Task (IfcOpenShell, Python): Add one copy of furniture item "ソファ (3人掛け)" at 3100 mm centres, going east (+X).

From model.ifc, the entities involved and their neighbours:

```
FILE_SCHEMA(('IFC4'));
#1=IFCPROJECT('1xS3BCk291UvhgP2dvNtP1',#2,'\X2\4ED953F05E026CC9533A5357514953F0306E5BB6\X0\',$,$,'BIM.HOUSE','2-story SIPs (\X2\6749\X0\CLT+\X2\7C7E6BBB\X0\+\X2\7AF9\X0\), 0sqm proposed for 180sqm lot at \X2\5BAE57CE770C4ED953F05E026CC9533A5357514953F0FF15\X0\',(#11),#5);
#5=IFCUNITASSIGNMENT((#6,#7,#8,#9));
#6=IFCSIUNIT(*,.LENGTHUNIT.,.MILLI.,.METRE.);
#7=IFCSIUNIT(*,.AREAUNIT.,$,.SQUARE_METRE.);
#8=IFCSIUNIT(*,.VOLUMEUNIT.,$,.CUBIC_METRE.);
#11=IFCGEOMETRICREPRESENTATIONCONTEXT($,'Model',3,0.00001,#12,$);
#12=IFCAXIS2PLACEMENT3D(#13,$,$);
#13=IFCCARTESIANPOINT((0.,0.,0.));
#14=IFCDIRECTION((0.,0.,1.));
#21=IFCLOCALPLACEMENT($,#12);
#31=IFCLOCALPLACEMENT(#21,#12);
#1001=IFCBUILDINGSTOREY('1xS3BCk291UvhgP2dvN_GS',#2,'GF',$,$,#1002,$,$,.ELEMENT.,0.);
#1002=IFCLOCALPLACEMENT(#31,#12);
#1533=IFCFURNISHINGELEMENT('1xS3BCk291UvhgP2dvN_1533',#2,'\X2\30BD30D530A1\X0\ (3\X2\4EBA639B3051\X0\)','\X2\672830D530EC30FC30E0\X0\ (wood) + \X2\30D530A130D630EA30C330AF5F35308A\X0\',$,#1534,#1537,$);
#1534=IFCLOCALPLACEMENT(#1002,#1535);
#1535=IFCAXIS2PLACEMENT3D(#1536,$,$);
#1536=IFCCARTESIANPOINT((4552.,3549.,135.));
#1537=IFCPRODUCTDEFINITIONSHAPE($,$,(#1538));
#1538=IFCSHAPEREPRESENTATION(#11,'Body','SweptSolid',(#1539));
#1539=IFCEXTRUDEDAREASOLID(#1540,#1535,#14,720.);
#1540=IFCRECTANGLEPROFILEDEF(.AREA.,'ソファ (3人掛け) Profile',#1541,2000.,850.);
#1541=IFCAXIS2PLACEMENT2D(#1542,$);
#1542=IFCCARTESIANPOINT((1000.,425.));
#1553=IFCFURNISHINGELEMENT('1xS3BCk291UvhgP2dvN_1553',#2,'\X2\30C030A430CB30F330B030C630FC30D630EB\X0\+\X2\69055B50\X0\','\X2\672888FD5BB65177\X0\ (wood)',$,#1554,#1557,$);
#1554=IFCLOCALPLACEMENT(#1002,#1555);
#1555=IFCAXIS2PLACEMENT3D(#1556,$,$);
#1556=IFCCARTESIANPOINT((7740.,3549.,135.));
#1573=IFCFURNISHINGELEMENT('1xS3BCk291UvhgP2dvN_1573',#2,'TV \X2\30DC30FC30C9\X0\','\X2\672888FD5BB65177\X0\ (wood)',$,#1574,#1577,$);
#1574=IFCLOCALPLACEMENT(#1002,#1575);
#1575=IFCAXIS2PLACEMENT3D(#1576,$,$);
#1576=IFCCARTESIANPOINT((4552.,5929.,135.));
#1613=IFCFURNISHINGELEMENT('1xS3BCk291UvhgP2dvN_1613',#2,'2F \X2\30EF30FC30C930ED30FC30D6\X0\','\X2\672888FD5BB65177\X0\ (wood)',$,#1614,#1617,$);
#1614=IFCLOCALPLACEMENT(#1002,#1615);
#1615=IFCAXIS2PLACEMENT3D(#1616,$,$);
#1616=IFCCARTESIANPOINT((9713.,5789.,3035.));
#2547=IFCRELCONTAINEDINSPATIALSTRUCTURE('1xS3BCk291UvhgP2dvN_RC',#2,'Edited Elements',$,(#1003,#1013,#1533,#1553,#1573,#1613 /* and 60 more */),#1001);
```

```python
import numpy as np
import ifcopenshell
import ifcopenshell.api.geometry
import ifcopenshell.api.root
import ifcopenshell.util.element
import ifcopenshell.util.placement

model = ifcopenshell.open("model.ifc")


def reuse_history(source, copy):
    """copy_class also copies each property set's owner history, people and application; keep the originals."""
    for rel in copy.IsDefinedBy:
        if rel.is_a("IfcRelDefinesByProperties") and (history := rel.RelatingPropertyDefinition.OwnerHistory):
            rel.RelatingPropertyDefinition.OwnerHistory = source.OwnerHistory
            ifcopenshell.util.element.remove_deep2(model, history)


source = model.by_id(1533)
base = ifcopenshell.util.placement.get_local_placement(source.ObjectPlacement)
step = np.array([1.0, 0.0, 0.0]) * 3100.0

for i in range(1, 2):
    copy = ifcopenshell.api.root.copy_class(model, product=source)
    copy.Representation = ifcopenshell.util.element.copy_deep(
        model, source.Representation, exclude=["IfcGeometricRepresentationContext", "IfcRepresentationMap"]
    )
    reuse_history(source, copy)
    matrix = base.copy()
    matrix[:3, 3] += i * step
    print("added at", matrix[:3, 3].round(3) + 0.0)
    ifcopenshell.api.geometry.edit_object_placement(model, product=copy, matrix=matrix, is_si=False)

model.write("model_updated.ifc")
```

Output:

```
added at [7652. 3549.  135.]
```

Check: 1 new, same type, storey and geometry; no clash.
